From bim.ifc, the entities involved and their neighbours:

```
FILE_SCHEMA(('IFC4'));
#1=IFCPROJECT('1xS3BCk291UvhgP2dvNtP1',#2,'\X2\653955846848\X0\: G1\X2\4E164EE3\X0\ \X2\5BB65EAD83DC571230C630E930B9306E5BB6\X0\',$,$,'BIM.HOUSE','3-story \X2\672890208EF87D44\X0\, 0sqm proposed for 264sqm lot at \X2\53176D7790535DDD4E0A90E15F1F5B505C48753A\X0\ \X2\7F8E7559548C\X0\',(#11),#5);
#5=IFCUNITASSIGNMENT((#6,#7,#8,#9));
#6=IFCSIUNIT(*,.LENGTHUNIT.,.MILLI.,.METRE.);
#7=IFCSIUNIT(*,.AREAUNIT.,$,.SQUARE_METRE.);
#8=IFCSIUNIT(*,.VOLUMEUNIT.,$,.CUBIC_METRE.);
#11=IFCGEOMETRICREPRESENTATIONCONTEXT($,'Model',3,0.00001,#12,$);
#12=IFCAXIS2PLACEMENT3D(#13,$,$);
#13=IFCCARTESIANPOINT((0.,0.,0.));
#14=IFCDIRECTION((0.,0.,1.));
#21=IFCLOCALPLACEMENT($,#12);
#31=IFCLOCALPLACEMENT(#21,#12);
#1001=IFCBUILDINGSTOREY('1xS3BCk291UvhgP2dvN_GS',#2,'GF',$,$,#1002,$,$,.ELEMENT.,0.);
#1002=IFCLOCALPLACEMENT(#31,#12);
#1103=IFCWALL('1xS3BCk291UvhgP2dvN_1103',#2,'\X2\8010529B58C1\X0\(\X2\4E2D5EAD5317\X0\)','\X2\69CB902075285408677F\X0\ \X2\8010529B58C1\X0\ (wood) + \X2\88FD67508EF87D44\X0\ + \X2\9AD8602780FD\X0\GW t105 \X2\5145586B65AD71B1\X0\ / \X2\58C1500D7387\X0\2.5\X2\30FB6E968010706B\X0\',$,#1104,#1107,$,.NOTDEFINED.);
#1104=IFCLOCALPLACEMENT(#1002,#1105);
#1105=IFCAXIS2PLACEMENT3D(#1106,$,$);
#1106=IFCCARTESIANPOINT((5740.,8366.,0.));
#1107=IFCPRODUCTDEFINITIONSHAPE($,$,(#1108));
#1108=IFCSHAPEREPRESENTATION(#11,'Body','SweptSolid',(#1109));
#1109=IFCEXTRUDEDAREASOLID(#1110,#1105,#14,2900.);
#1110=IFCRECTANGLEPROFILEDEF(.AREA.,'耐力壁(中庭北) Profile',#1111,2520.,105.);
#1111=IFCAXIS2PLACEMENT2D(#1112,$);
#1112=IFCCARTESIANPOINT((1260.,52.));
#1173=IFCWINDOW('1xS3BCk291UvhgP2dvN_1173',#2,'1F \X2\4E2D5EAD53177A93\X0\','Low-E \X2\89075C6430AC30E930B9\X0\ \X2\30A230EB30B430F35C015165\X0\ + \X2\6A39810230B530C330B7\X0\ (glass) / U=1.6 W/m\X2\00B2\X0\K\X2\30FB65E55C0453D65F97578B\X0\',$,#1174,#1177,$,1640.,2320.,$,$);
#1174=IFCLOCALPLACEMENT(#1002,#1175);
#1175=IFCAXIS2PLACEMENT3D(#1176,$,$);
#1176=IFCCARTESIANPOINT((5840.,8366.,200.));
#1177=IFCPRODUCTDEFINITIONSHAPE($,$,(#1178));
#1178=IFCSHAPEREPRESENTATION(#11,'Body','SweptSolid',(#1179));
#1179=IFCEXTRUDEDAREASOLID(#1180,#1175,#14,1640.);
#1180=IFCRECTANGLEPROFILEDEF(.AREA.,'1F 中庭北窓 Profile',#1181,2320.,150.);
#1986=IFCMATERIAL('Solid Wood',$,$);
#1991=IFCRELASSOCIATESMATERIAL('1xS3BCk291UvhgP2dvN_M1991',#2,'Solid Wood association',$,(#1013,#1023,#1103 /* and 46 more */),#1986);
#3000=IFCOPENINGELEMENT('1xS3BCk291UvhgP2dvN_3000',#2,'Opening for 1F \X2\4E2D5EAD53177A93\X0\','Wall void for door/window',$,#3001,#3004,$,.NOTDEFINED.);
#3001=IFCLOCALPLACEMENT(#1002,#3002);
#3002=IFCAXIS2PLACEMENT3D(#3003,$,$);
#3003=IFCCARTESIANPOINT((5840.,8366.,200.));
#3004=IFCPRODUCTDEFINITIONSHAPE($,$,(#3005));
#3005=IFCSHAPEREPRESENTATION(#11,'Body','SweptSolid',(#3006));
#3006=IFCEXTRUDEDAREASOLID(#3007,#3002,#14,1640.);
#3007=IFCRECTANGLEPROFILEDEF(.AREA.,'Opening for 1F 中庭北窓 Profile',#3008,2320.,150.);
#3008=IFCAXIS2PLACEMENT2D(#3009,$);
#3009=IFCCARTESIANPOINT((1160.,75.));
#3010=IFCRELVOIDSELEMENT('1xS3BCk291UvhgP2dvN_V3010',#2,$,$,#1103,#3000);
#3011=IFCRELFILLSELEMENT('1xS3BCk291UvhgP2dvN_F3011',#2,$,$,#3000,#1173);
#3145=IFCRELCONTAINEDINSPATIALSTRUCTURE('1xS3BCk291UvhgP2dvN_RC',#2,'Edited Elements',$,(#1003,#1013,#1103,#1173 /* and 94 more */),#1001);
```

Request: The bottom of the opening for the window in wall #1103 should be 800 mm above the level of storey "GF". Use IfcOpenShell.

```python
import numpy as np
import ifcopenshell
import ifcopenshell.api.geometry
import ifcopenshell.geom
import ifcopenshell.util.element
import ifcopenshell.util.placement
import ifcopenshell.util.shape
import ifcopenshell.util.unit

model = ifcopenshell.open("bim.ifc")
unit_scale = ifcopenshell.util.unit.calculate_unit_scale(model)

window = model.by_guid("1xS3BCk291UvhgP2dvN_1173")
opening = window.FillsVoids[0].RelatingOpeningElement
storey = ifcopenshell.util.element.get_container(window, ifc_class="IfcBuildingStorey")
level = ifcopenshell.util.placement.get_local_placement(storey.ObjectPlacement)[2, 3]

# The opening's origin need not be at the sill, so measure its lowest point.
shape = ifcopenshell.geom.create_shape(ifcopenshell.geom.settings(), opening)
bottom = ifcopenshell.util.shape.get_shape_bottom_elevation(shape, shape.geometry) / unit_scale
dz = level + 0.8 / unit_scale - bottom

shift = np.array([0.0, 0.0, dz])
# The window is not placed relative to its opening, so move both.
for product in (opening, window):
    matrix = ifcopenshell.util.placement.get_local_placement(product.ObjectPlacement)
    matrix[:3, 3] += shift
    ifcopenshell.api.geometry.edit_object_placement(model, product=product, matrix=matrix, is_si=False)

print(f"moved by {dz * unit_scale:+.3f} m")

model.write("bim_rev.ifc")
```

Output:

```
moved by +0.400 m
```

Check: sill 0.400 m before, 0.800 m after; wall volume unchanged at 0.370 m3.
